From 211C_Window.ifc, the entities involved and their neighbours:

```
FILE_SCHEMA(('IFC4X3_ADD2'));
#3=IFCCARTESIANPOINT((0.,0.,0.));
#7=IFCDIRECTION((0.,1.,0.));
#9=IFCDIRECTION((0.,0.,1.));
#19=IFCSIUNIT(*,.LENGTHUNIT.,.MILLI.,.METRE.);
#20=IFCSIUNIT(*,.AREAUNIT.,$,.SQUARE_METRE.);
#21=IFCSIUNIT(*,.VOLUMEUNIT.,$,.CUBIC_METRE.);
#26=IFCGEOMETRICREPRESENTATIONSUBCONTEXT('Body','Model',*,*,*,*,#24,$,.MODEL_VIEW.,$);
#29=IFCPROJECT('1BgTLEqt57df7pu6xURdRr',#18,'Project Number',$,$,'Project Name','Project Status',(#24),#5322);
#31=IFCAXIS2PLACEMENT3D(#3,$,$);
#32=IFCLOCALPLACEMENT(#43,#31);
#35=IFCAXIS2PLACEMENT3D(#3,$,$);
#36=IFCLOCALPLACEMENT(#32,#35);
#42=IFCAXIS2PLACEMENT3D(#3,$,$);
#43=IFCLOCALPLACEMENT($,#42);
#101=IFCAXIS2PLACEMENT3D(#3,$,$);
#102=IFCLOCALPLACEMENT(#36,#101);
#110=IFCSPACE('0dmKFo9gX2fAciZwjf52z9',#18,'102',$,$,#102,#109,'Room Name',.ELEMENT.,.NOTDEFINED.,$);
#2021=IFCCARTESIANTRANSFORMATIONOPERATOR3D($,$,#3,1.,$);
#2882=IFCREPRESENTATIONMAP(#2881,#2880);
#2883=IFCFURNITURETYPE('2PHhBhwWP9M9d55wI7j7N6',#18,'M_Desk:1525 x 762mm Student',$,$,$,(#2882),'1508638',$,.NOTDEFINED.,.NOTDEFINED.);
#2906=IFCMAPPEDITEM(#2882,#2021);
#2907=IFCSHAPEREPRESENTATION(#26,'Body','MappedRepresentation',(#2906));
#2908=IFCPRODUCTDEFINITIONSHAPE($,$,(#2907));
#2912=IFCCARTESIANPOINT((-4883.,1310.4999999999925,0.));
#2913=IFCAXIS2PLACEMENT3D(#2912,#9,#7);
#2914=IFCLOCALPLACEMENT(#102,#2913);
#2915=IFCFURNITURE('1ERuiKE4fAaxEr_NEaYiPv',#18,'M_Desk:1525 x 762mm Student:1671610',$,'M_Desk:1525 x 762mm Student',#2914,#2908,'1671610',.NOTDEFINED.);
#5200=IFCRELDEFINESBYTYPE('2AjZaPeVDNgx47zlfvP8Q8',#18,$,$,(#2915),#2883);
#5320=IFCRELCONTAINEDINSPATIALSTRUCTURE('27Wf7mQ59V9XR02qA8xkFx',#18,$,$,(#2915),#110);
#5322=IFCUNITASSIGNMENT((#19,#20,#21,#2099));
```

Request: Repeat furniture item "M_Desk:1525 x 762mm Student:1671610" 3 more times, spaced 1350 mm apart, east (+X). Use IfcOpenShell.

```python
import numpy as np
import ifcopenshell
import ifcopenshell.api.geometry
import ifcopenshell.api.root
import ifcopenshell.util.element
import ifcopenshell.util.placement
import ifcopenshell.util.unit

model = ifcopenshell.open("211C_Window.ifc")
unit_scale = ifcopenshell.util.unit.calculate_unit_scale(model)


def reuse_history(source, copy):
    """copy_class also copies each property set's owner history, people and application; keep the originals."""
    for rel in copy.IsDefinedBy:
        if rel.is_a("IfcRelDefinesByProperties") and (history := rel.RelatingPropertyDefinition.OwnerHistory):
            rel.RelatingPropertyDefinition.OwnerHistory = source.OwnerHistory
            ifcopenshell.util.element.remove_deep2(model, history)


source = model.by_id(2915)
base = ifcopenshell.util.placement.get_local_placement(source.ObjectPlacement)
step = np.array([1.0, 0.0, 0.0]) * 1.35 / unit_scale

for i in range(1, 4):
    copy = ifcopenshell.api.root.copy_class(model, product=source)
    copy.Representation = ifcopenshell.util.element.copy_deep(
        model, source.Representation, exclude=["IfcGeometricRepresentationContext", "IfcRepresentationMap"]
    )
    copy.Name = "M_Desk:1525 x 762mm Student"
    copy.Tag = None
    reuse_history(source, copy)
    matrix = base.copy()
    matrix[:3, 3] += i * step
    print("added at", matrix[:3, 3].round(3) + 0.0)
    ifcopenshell.api.geometry.edit_object_placement(model, product=copy, matrix=matrix, is_si=False)

model.write("211C_Window-out.ifc")
```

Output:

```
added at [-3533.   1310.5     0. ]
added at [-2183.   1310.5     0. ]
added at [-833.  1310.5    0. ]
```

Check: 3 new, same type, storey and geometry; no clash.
